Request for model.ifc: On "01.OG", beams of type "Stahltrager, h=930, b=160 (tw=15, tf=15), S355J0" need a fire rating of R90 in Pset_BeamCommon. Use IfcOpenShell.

First a look at what the model holds.

```python
import ifcopenshell
import ifcopenshell.util.element

model = ifcopenshell.open("model.ifc")
print(model.schema)
storey = next(s for s in model.by_type("IfcBuildingStorey") if s.Name == "01.OG")
beams = [e for e in ifcopenshell.util.element.get_decomposition(storey) if e.is_a("IfcBeam")]
seen = {}
for e in beams:
    element_type = ifcopenshell.util.element.get_type(e)
    key = (element_type.Name if element_type != e and element_type else None, ifcopenshell.util.element.get_pset(e, "Pset_BeamCommon", "FireRating"))
    seen[key] = seen.get(key, 0) + 1
for (name, value), count in sorted(seen.items(), key=str):
    print(count, "x", name, "|", value)
```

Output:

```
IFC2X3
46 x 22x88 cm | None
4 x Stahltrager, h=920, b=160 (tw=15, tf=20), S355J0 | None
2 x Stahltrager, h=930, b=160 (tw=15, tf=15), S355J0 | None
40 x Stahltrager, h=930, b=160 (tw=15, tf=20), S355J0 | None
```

```python
import ifcopenshell
import ifcopenshell.api.pset
import ifcopenshell.util.element

model = ifcopenshell.open("model.ifc")

storey = next(s for s in model.by_type("IfcBuildingStorey") if s.Name == "01.OG")
beams = [e for e in ifcopenshell.util.element.get_decomposition(storey) if e.is_a("IfcBeam")]

count = 0
for e in beams:
    element_type = ifcopenshell.util.element.get_type(e)
    if element_type in (None, e) or element_type.Name != "Stahltrager, h=930, b=160 (tw=15, tf=15), S355J0":
        continue
    # add_pset returns the element's existing set when there is one.
    pset = ifcopenshell.api.pset.add_pset(model, product=e, name="Pset_BeamCommon")
    ifcopenshell.api.pset.edit_pset(model, pset=pset, properties={"FireRating": "R90"})
    count += 1

print(count, "beams updated")

model.write("model_v2.ifc")
```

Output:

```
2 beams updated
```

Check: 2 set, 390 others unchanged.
